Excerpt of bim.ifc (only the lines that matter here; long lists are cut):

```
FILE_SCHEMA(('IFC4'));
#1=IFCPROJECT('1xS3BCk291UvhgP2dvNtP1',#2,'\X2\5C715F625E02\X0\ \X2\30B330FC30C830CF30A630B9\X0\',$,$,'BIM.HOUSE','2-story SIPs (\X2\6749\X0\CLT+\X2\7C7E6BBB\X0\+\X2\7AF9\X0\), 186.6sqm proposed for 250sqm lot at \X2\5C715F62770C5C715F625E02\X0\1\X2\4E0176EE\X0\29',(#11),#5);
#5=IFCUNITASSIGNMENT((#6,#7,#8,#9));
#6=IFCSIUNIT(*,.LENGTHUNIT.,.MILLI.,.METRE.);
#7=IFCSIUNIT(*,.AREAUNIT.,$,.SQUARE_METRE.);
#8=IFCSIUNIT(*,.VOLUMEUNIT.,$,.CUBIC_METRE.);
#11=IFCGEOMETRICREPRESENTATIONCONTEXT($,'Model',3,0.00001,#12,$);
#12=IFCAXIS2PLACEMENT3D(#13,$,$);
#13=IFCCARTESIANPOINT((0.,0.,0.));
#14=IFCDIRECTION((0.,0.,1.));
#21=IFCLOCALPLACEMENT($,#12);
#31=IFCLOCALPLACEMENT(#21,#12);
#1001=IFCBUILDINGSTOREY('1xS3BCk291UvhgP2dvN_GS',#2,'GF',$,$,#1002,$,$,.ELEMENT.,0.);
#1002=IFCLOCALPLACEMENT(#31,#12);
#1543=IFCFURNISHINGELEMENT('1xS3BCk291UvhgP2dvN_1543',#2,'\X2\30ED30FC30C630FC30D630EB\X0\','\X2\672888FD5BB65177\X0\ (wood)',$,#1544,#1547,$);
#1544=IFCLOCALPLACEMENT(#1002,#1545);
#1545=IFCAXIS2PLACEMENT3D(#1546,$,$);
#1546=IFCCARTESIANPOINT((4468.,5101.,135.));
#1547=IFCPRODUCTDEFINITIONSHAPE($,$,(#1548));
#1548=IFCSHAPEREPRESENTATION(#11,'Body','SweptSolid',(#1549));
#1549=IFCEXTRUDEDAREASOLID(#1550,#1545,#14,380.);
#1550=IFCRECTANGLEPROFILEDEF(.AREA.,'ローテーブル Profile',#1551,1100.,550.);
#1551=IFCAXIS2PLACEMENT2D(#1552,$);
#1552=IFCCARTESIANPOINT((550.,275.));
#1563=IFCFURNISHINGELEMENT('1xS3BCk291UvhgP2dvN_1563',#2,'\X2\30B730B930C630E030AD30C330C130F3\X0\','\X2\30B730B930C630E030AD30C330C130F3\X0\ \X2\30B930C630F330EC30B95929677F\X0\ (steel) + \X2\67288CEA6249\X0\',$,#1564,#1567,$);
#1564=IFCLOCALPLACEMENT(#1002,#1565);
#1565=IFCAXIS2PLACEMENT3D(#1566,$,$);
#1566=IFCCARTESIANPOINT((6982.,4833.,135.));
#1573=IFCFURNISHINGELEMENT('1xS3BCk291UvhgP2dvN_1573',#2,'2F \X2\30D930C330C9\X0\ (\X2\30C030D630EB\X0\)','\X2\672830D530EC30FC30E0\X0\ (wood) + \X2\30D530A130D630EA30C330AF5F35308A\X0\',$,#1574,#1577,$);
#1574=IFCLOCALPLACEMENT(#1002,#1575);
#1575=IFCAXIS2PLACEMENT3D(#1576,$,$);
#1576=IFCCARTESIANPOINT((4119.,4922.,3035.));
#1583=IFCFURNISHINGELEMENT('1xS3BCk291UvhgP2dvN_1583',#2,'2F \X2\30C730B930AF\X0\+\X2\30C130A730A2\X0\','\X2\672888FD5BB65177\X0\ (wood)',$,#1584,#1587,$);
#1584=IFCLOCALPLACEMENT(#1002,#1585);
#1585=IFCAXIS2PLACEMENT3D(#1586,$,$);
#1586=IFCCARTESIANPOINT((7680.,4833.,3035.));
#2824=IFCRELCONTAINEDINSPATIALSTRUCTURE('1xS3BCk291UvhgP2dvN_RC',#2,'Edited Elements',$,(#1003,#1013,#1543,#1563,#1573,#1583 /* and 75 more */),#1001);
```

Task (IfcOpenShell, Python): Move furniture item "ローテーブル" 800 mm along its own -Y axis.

```python
import ifcopenshell
import ifcopenshell.api.geometry
import ifcopenshell.util.placement

model = ifcopenshell.open("bim.ifc")

item = model.by_id(1543)
matrix = ifcopenshell.util.placement.get_local_placement(item.ObjectPlacement)
matrix[:3, 3] -= matrix[:3, 1] * 800.0
ifcopenshell.api.geometry.edit_object_placement(model, product=item, matrix=matrix, is_si=False)

print(ifcopenshell.util.placement.get_local_placement(item.ObjectPlacement).round(3) + 0.0)

model.write("bim_v2.ifc")
```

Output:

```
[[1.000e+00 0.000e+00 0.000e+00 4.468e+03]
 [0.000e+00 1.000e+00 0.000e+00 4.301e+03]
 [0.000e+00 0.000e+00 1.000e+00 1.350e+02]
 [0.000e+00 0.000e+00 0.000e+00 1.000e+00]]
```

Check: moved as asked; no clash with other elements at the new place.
